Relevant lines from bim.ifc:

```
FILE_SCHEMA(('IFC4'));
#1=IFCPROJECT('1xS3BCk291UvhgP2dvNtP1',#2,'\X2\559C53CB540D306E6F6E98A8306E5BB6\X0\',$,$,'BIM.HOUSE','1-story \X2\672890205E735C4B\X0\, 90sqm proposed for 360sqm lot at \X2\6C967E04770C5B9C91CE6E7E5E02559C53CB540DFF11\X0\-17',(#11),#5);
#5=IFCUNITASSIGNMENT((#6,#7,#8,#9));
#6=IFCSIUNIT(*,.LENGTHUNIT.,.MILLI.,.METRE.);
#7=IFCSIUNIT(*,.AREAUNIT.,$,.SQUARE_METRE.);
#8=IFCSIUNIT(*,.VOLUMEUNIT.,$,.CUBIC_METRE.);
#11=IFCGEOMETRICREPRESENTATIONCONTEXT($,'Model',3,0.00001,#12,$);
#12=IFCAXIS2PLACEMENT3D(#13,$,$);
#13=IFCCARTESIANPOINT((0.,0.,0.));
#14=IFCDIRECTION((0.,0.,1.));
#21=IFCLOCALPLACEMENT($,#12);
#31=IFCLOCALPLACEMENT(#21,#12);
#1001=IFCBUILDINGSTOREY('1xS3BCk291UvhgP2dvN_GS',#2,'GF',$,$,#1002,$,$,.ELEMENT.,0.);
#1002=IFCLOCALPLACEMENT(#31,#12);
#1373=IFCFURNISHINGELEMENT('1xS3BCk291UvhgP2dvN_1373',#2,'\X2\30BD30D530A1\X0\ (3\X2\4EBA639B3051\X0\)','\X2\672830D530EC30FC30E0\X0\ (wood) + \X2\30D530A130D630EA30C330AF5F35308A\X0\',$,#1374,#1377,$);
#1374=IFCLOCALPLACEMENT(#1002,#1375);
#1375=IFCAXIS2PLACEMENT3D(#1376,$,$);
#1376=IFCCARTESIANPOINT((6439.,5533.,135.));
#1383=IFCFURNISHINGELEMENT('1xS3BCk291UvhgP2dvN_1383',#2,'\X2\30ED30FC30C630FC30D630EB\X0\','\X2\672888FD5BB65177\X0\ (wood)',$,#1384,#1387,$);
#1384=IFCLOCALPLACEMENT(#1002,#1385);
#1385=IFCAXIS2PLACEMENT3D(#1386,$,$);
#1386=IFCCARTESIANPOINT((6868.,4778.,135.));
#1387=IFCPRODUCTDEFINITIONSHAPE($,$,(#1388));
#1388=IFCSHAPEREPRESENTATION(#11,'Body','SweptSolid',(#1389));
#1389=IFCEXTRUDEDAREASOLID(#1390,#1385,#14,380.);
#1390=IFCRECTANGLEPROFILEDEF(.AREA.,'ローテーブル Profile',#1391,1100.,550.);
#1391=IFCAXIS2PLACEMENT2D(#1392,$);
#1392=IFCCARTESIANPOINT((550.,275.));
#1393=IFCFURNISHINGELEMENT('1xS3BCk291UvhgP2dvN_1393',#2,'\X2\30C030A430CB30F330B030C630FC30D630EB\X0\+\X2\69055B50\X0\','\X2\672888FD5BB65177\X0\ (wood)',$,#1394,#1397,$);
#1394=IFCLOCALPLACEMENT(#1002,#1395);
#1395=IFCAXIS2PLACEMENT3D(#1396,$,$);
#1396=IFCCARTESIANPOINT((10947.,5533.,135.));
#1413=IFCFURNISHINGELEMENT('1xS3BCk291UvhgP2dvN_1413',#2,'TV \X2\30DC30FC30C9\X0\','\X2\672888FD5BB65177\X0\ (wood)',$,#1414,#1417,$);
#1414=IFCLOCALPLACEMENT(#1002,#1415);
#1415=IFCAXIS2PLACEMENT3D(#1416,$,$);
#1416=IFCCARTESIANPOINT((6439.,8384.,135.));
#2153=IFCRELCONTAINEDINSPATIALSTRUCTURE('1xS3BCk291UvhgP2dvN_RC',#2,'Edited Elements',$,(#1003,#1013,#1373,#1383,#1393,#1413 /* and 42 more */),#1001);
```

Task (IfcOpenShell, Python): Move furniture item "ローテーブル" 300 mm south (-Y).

```python
import ifcopenshell
import ifcopenshell.api.geometry
import ifcopenshell.util.placement
import ifcopenshell.util.unit

model = ifcopenshell.open("bim.ifc")
unit_scale = ifcopenshell.util.unit.calculate_unit_scale(model)

item = model.by_id(1383)
matrix = ifcopenshell.util.placement.get_local_placement(item.ObjectPlacement)
matrix[1, 3] -= 0.3 / unit_scale
ifcopenshell.api.geometry.edit_object_placement(model, product=item, matrix=matrix, is_si=False)

print(ifcopenshell.util.placement.get_local_placement(item.ObjectPlacement).round(3) + 0.0)

model.write("bim-out.ifc")
```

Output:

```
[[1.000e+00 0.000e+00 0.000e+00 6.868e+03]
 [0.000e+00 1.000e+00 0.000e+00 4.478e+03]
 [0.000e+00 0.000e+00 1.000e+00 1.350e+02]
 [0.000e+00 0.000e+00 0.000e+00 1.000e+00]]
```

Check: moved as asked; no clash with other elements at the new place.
